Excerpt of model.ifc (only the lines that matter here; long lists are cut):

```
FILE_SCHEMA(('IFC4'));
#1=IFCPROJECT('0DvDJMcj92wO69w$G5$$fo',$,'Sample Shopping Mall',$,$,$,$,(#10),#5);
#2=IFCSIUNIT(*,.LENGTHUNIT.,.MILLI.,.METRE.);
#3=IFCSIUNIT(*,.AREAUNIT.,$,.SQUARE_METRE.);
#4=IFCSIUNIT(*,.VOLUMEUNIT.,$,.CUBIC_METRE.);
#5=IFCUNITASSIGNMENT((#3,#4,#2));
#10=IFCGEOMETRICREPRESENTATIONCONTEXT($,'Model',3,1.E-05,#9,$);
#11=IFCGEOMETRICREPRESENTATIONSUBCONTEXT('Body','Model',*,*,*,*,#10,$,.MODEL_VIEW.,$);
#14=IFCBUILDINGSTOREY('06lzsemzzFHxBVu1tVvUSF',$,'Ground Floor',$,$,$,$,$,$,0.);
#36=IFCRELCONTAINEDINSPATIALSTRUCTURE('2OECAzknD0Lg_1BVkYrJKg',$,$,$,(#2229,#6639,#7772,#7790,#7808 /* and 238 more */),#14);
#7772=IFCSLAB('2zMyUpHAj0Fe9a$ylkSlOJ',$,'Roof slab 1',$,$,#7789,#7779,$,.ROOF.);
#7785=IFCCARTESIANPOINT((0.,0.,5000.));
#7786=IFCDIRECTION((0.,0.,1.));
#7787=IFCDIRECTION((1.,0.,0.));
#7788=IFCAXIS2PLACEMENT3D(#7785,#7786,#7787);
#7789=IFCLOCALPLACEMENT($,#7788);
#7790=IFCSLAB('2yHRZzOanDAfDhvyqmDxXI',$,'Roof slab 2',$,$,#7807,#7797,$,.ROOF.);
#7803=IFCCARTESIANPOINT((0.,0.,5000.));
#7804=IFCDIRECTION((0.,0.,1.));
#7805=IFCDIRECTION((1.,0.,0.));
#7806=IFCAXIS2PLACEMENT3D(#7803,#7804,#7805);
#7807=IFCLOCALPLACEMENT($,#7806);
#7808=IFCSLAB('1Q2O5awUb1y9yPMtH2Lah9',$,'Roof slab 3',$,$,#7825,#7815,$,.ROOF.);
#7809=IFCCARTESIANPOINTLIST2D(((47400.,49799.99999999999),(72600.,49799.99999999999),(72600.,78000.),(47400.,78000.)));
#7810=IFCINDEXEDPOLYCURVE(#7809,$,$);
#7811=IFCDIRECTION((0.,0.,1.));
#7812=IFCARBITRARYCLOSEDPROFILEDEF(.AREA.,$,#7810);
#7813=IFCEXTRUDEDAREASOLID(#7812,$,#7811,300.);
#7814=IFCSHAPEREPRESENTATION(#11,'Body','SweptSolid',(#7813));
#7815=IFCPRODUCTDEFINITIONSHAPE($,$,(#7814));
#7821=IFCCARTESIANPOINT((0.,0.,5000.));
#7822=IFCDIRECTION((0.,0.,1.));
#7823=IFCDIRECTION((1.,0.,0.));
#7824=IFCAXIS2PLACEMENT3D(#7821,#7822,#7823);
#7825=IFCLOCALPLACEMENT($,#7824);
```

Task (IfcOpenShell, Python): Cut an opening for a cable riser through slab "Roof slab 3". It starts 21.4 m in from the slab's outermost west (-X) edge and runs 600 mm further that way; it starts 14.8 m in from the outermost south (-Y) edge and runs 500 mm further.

```python
import numpy as np
import ifcopenshell
import ifcopenshell.api.feature
import ifcopenshell.api.geometry
import ifcopenshell.api.root
import ifcopenshell.geom
import ifcopenshell.util.placement
import ifcopenshell.util.representation
import ifcopenshell.util.shape
import ifcopenshell.util.unit

model = ifcopenshell.open("model.ifc")
unit_scale = ifcopenshell.util.unit.calculate_unit_scale(model)
settings = ifcopenshell.geom.settings()


def volume(element):
    """Net volume in cubic metres, openings subtracted."""
    shape = ifcopenshell.geom.create_shape(settings, element)
    return ifcopenshell.util.shape.get_volume(shape.geometry)


slab = model.by_id(7808)
before = volume(slab)

# Extent in the slab's own axes, in metres. The edges named are its -X and -Y sides.
slab_shape = ifcopenshell.geom.create_shape(settings, slab)
vertices = ifcopenshell.util.shape.get_vertices(slab_shape.geometry)
x_min, y_min, bottom = vertices.min(axis=0)
top = vertices[:, 2].max()

opening = ifcopenshell.api.root.create_entity(model, ifc_class="IfcOpeningElement", name="Cable riser opening", predefined_type="OPENING")
context = ifcopenshell.util.representation.get_context(model, "Model", "Body", "MODEL_VIEW")
width, depth = 0.6, 0.5
outline = [(0.0, 0.0), (width, 0.0), (width, depth), (0.0, depth), (0.0, 0.0)]
# Overshoot both faces by 50 mm so the cut is clean.
shape = ifcopenshell.api.geometry.add_slab_representation(
    model, context=context, depth=top - bottom + 0.1, polyline=outline
)
ifcopenshell.api.geometry.assign_representation(model, product=opening, representation=shape)

matrix = ifcopenshell.util.placement.get_local_placement(slab.ObjectPlacement)
matrix[:, 3] = matrix @ np.append(np.array([x_min + 21.4, y_min + 14.8, bottom - 0.05]) / unit_scale, 1.0)
ifcopenshell.api.geometry.edit_object_placement(model, product=opening, matrix=matrix, is_si=False)
ifcopenshell.api.feature.add_feature(model, feature=opening, element=slab)

after = volume(slab)

print(f"slab volume {before:.3f} -> {after:.3f} m3")

model.write("model_edited.ifc")
```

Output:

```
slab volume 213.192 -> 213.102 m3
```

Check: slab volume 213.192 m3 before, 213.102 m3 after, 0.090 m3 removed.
